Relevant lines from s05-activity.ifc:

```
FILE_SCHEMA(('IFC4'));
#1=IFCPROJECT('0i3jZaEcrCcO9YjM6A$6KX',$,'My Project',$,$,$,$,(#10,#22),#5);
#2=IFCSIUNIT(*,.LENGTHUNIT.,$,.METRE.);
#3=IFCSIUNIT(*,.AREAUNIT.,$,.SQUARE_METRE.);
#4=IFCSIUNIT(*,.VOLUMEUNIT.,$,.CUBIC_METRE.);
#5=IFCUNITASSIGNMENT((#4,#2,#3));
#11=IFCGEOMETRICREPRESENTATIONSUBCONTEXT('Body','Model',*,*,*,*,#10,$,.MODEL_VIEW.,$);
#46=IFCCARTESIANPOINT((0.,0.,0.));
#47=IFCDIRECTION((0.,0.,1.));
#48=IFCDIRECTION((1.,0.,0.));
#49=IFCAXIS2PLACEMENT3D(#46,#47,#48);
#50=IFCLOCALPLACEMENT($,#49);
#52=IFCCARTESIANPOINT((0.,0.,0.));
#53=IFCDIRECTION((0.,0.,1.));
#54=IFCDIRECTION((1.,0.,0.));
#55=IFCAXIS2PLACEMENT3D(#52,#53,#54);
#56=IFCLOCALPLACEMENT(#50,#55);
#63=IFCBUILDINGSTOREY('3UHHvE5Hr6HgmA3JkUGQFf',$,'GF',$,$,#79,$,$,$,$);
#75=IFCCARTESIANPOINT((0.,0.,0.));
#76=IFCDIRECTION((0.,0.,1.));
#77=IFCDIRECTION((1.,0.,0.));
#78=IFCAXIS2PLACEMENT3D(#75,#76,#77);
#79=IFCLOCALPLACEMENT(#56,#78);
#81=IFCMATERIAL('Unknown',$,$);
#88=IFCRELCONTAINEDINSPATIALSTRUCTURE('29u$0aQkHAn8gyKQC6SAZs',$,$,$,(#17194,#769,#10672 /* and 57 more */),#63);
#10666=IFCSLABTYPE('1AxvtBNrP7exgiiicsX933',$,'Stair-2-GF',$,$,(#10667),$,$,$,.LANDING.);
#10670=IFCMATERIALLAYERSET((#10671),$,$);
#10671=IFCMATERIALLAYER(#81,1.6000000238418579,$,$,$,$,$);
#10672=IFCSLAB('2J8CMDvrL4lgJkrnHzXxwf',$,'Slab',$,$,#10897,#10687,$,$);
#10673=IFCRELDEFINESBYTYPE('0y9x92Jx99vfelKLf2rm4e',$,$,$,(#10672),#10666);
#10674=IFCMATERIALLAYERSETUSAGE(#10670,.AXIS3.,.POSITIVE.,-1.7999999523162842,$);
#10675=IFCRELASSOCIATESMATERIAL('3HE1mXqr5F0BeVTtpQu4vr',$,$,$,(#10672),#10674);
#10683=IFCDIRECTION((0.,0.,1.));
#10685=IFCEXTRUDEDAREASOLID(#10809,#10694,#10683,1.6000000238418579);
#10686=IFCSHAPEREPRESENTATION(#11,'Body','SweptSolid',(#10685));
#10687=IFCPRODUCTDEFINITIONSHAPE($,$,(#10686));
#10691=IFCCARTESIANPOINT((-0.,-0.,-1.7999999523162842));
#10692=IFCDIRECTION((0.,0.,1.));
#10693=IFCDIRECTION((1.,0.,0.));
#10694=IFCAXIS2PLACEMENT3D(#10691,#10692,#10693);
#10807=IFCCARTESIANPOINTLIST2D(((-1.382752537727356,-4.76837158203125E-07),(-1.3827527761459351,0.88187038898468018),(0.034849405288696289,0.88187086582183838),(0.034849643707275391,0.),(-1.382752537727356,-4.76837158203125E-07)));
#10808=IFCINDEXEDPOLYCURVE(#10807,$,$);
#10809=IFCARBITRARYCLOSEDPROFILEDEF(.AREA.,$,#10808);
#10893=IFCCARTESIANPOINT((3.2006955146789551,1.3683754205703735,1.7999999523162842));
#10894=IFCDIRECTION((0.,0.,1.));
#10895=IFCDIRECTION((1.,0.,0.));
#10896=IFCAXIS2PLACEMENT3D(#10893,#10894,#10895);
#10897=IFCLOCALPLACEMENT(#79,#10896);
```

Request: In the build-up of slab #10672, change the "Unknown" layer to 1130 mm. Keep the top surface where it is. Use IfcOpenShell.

```python
import ifcopenshell
import ifcopenshell.util.element
import ifcopenshell.util.representation
import ifcopenshell.util.unit

model = ifcopenshell.open("s05-activity.ifc")
unit_scale = ifcopenshell.util.unit.calculate_unit_scale(model)

layer_set = model.by_id(10670)
layer = next(l for l in layer_set.MaterialLayers if l.Material and l.Material.Name == "Unknown")
change = 1.13 / unit_scale - layer.LayerThickness
layer.LayerThickness += change

# Geometry does not follow the layer set by itself.
slabs = [e for e in ifcopenshell.util.element.get_elements_by_material(model, layer_set) if e.is_a("IfcSlab")]
for slab in sorted(slabs, key=lambda e: e.id()):
    body = ifcopenshell.util.representation.get_representation(slab, "Model", "Body")
    solid = body.Items[0]
    old_depth = solid.Depth
    solid.Depth += change
    # Extruded upwards: lower the start of the extrusion so the top stays.
    x, y, z = solid.Position.Location.Coordinates
    solid.Position.Location = model.createIfcCartesianPoint((x, y, z - change))
    print(slab.id(), f"{old_depth:g} -> {solid.Depth:g}")

# The layers are counted up from the underside, which has moved.
for usage in {ifcopenshell.util.element.get_material(slab) for slab in slabs}:
    usage.OffsetFromReferenceLine -= change

model.write("s05-activity_updated.ifc")
```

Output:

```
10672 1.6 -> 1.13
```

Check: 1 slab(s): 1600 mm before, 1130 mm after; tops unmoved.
